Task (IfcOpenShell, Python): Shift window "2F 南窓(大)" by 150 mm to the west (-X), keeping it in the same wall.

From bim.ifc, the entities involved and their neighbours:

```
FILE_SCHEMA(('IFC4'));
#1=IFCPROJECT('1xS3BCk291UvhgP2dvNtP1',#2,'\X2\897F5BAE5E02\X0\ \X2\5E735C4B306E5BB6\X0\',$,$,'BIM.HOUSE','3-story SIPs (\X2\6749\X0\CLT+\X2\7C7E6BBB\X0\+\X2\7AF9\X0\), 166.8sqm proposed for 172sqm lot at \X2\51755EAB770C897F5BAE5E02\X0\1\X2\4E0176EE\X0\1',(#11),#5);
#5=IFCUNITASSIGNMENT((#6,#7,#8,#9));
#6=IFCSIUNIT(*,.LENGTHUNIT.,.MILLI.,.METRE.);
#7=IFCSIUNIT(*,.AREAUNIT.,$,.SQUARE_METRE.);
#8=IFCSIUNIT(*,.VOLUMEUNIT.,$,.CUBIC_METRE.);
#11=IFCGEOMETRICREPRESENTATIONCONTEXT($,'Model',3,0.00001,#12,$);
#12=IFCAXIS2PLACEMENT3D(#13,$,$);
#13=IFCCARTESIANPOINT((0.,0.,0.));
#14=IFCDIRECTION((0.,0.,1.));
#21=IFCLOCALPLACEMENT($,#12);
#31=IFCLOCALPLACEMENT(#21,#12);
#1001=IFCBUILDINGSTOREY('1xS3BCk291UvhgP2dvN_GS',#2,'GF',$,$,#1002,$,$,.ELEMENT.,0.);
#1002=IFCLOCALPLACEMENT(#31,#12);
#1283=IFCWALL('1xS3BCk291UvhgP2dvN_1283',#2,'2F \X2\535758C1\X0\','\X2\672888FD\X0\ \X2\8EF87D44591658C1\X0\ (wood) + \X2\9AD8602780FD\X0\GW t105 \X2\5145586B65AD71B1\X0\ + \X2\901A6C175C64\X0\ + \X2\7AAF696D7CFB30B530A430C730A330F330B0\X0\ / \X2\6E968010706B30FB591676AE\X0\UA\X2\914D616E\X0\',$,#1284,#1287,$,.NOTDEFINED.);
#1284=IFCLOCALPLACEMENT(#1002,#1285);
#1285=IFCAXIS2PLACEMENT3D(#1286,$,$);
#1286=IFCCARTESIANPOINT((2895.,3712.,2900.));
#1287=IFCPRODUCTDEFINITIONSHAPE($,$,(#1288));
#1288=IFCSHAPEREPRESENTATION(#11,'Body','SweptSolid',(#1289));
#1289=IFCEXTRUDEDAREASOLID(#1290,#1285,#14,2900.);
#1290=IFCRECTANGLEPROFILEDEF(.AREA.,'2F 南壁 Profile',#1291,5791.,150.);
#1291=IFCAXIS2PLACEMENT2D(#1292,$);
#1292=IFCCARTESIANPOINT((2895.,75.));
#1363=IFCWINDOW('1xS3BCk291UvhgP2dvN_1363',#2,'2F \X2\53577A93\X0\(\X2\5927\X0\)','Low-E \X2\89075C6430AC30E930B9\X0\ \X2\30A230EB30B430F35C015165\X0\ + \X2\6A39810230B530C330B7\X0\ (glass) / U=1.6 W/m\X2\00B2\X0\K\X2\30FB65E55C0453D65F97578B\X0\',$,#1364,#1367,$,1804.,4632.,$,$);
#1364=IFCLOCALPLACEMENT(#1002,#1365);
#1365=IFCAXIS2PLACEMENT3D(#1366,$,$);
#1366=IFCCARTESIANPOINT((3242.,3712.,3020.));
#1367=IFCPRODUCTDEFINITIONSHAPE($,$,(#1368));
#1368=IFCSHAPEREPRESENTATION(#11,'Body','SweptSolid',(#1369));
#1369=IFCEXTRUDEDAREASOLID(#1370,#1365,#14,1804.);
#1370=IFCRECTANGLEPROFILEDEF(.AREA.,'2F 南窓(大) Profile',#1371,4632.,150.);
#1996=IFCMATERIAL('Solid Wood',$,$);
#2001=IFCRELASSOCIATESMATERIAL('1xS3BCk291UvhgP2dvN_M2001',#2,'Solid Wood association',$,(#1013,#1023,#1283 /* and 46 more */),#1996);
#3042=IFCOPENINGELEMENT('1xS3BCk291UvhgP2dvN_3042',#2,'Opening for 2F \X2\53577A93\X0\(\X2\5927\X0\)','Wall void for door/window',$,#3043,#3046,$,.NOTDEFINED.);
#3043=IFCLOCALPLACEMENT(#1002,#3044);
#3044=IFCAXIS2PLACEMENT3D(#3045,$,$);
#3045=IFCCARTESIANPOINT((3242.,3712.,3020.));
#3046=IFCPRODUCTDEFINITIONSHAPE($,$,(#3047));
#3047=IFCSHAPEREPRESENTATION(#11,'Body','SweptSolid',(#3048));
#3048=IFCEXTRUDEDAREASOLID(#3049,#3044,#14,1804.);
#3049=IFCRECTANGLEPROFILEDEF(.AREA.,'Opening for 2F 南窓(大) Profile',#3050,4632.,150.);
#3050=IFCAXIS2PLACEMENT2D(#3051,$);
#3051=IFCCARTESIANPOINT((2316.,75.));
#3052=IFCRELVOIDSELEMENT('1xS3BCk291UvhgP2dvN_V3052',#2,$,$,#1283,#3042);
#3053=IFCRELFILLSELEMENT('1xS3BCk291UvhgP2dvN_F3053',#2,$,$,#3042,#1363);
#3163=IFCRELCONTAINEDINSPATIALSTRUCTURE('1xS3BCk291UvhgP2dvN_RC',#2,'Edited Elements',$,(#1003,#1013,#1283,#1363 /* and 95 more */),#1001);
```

```python
import ifcopenshell
import ifcopenshell.api.geometry
import ifcopenshell.util.placement

model = ifcopenshell.open("bim.ifc")

window = model.by_guid("1xS3BCk291UvhgP2dvN_1363")
opening = window.FillsVoids[0].RelatingOpeningElement
wall = opening.VoidsElements[0].RelatingBuildingElement

wall_matrix = ifcopenshell.util.placement.get_local_placement(wall.ObjectPlacement)
shift = wall_matrix[:3, 0] * -150.0
before = ifcopenshell.util.placement.get_local_placement(window.ObjectPlacement)[:3, 3].copy()

# The window is not placed relative to its opening, so move both.
for product in (opening, window):
    matrix = ifcopenshell.util.placement.get_local_placement(product.ObjectPlacement)
    matrix[:3, 3] += shift
    ifcopenshell.api.geometry.edit_object_placement(model, product=product, matrix=matrix, is_si=False)

after = ifcopenshell.util.placement.get_local_placement(window.ObjectPlacement)[:3, 3]
print("window moved by", (after - before).round(3) + 0.0)

model.write("bim-out.ifc")
```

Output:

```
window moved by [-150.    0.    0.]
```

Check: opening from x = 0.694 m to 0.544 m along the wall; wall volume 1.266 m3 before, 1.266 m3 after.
